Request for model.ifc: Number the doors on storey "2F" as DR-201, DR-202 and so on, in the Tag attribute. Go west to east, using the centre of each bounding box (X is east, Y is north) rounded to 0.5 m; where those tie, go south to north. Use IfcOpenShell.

First a look at what the model holds.

```python
import ifcopenshell
import ifcopenshell.util.element
import ifcopenshell.util.placement

model = ifcopenshell.open("model.ifc")
print(model.schema)
storey = next(s for s in model.by_type("IfcBuildingStorey") if s.Name == "2F")
doors = [e for e in ifcopenshell.util.element.get_decomposition(storey) if e.is_a("IfcDoor")]
for e in sorted(doors, key=lambda e: e.id()):
    origin = ifcopenshell.util.placement.get_local_placement(e.ObjectPlacement)[:3, 3]
    print(e.id(), e.Tag, e.Name, origin.round(2) + 0.0, sep=" | ")
```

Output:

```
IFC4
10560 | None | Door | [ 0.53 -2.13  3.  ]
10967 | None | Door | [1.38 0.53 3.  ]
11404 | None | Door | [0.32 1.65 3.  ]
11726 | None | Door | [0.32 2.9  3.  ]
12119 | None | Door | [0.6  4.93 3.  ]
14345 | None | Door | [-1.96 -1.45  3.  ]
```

```python
import ifcopenshell
import ifcopenshell.geom
import ifcopenshell.util.element
import ifcopenshell.util.shape

model = ifcopenshell.open("model.ifc")
settings = ifcopenshell.geom.settings()
settings.set("use-world-coords", True)


def centre(element):
    shape = ifcopenshell.geom.create_shape(settings, element)
    return ifcopenshell.util.shape.get_bbox_centroid(shape.geometry)


storey = next(s for s in model.by_type("IfcBuildingStorey") if s.Name == "2F")
doors = [e for e in ifcopenshell.util.element.get_decomposition(storey) if e.is_a("IfcDoor")]

# Insertion points can sit at a corner or the storey origin, so sort by the geometry (in metres).
centres = {e: centre(e) for e in doors}
doors.sort(key=lambda e: (round(centres[e][0] / 0.5), centres[e][1]))

for i, e in enumerate(doors, start=1):
    number = f"DR-2{i:02d}"
    e.Tag = number
    print(e.id(), number)

model.write("model-out.ifc")
```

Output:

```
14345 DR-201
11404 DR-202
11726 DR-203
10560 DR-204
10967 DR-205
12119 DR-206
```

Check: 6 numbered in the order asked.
